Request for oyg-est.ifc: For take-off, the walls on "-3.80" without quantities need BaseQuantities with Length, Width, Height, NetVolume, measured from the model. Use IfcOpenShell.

First a look at what the model holds.

```python
import ifcopenshell
import ifcopenshell.util.element
import ifcopenshell.util.unit

model = ifcopenshell.open("oyg-est.ifc")
print(model.schema)
for unit_type in ("LENGTHUNIT", "AREAUNIT", "VOLUMEUNIT"):
    print(unit_type, ifcopenshell.util.unit.calculate_unit_scale(model, unit_type))
storey = next(s for s in model.by_type("IfcBuildingStorey") if s.Name == "-3.80")
walls = [e for e in ifcopenshell.util.element.get_decomposition(storey) if e.is_a("IfcWall")]
for e in sorted(walls, key=lambda e: e.id()):
    print(e.id(), e.is_a(), e.Name, list(ifcopenshell.util.element.get_psets(e, qtos_only=True)), sep=" | ")
```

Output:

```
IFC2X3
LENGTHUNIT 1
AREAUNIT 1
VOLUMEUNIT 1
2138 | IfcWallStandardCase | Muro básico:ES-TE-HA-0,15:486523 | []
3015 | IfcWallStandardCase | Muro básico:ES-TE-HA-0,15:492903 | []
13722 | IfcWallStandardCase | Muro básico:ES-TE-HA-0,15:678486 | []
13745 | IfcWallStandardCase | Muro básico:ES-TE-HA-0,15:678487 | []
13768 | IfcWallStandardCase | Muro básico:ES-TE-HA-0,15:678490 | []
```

```python
import ifcopenshell
import ifcopenshell.api.pset
import ifcopenshell.geom
import ifcopenshell.util.element
import ifcopenshell.util.shape
import ifcopenshell.util.unit

model = ifcopenshell.open("oyg-est.ifc")
unit_scale = ifcopenshell.util.unit.calculate_unit_scale(model)
volume_scale = ifcopenshell.util.unit.calculate_unit_scale(model, "VOLUMEUNIT")
settings = ifcopenshell.geom.settings()

storey = next(s for s in model.by_type("IfcBuildingStorey") if s.Name == "-3.80")
walls = [e for e in ifcopenshell.util.element.get_decomposition(storey) if e.is_a("IfcWall")]

for e in sorted(walls, key=lambda e: e.id()):
    if ifcopenshell.util.element.get_psets(e, qtos_only=True, should_inherit=False):
        continue
    # Geometry comes back in metres, in the element's own axes.
    shape = ifcopenshell.geom.create_shape(settings, e)
    values = {
        "Length": ifcopenshell.util.shape.get_x(shape.geometry) / unit_scale,
        "Width": ifcopenshell.util.shape.get_y(shape.geometry) / unit_scale,
        "Height": ifcopenshell.util.shape.get_z(shape.geometry) / unit_scale,
        "NetVolume": ifcopenshell.util.shape.get_volume(shape.geometry) / volume_scale,
    }
    qto = ifcopenshell.api.pset.add_qto(model, product=e, name="BaseQuantities")
    ifcopenshell.api.pset.edit_qto(model, qto=qto, properties=values)
    print(e.id(), {k: round(v, 3) for k, v in values.items()})

model.write("oyg-est_v2.ifc")
```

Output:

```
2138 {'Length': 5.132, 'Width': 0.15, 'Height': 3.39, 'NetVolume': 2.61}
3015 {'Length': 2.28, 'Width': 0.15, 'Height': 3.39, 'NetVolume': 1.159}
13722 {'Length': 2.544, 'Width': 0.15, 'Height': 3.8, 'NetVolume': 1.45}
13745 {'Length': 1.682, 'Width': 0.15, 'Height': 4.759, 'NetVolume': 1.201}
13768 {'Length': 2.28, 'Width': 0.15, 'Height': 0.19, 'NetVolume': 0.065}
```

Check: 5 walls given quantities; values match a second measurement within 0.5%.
